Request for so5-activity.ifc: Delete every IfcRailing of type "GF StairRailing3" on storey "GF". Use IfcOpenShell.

First a look at what the model holds.

```python
import ifcopenshell
import ifcopenshell.util.element

model = ifcopenshell.open("so5-activity.ifc")
print(model.schema)
storey = next(s for s in model.by_type("IfcBuildingStorey") if s.Name == "GF")
railings = [e for e in ifcopenshell.util.element.get_decomposition(storey) if e.is_a("IfcRailing")]
seen = {}
for e in railings:
    element_type = ifcopenshell.util.element.get_type(e)
    name = element_type.Name if element_type not in (None, e) else None
    seen[name] = seen.get(name, 0) + 1
for name, count in sorted(seen.items(), key=str):
    print(count, "x", name)
```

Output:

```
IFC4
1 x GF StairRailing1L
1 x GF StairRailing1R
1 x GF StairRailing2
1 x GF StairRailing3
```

```python
import ifcopenshell
import ifcopenshell.api.root
import ifcopenshell.util.element

model = ifcopenshell.open("so5-activity.ifc")

storey = next(s for s in model.by_type("IfcBuildingStorey") if s.Name == "GF")
railings = [e for e in ifcopenshell.util.element.get_decomposition(storey) if e.is_a("IfcRailing")]
targets = [e for e in railings if (t := ifcopenshell.util.element.get_type(e)) not in (None, e) and t.Name == "GF StairRailing3"]

for e in targets:
    ifcopenshell.api.root.remove_product(model, product=e)
print(len(targets), "removed")

model.write("so5-activity_edited.ifc")
```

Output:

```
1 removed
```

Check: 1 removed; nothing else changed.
